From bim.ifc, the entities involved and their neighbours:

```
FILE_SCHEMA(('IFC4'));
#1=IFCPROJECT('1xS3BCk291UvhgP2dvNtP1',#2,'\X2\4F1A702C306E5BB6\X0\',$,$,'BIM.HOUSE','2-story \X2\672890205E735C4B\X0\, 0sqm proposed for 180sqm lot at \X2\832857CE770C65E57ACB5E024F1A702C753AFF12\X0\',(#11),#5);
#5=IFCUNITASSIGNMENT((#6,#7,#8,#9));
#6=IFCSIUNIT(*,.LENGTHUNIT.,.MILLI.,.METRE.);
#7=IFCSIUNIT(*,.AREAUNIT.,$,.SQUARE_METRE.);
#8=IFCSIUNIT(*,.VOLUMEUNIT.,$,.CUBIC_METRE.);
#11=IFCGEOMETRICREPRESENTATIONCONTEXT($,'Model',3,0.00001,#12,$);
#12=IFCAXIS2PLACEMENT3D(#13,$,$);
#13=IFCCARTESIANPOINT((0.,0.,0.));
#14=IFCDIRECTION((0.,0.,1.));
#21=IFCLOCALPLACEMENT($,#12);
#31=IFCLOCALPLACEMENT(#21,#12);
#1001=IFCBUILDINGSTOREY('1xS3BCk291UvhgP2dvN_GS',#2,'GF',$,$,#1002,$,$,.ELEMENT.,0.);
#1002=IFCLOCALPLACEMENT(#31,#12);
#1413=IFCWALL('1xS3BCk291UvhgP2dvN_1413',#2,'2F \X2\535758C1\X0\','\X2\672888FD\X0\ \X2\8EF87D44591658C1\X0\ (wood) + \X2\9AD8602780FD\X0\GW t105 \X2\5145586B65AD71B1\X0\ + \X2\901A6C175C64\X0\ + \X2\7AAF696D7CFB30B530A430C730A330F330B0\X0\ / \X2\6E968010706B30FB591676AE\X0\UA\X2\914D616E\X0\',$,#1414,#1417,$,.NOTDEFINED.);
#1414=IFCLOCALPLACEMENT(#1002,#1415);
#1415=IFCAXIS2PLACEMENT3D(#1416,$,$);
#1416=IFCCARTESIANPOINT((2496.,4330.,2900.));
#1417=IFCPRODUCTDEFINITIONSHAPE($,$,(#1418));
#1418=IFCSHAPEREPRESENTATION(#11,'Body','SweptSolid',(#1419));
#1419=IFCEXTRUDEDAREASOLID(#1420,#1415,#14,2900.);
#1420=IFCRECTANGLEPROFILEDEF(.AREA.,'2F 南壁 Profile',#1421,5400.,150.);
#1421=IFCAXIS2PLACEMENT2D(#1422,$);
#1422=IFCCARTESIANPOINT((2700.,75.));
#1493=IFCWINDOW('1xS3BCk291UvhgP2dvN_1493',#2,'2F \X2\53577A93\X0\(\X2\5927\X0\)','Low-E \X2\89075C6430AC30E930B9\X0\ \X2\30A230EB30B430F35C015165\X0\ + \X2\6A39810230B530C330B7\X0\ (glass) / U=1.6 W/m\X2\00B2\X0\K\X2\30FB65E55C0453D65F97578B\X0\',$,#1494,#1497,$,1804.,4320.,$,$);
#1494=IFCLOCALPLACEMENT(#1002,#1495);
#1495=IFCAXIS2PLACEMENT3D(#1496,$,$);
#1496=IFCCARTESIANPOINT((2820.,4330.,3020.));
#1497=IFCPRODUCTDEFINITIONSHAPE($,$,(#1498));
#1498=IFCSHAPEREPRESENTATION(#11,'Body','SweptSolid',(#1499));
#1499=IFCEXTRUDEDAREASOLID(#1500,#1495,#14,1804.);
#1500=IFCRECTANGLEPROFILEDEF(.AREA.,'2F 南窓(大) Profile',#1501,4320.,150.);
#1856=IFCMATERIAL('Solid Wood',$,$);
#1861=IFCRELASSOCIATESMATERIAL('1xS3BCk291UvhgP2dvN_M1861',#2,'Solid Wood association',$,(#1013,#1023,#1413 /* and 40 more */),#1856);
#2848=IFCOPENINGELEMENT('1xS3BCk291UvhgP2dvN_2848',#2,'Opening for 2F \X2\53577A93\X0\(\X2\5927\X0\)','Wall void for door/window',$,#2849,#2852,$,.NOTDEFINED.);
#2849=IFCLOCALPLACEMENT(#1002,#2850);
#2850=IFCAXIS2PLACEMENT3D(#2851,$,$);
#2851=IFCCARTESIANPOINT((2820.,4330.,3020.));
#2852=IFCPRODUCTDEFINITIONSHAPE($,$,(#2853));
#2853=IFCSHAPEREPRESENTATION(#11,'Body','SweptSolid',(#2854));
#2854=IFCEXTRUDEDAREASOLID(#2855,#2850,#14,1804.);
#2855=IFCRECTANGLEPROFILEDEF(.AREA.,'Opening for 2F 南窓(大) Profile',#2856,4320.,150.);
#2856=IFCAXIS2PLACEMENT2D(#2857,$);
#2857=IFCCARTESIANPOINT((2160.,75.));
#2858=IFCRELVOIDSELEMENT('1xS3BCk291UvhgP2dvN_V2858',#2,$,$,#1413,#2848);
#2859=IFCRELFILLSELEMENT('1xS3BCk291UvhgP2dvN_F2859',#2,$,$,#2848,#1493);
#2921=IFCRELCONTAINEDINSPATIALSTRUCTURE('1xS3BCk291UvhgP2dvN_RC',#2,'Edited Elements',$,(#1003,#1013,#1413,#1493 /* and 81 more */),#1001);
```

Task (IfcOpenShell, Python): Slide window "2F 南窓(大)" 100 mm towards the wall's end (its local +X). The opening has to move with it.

```python
import ifcopenshell
import ifcopenshell.api.geometry
import ifcopenshell.util.placement
import ifcopenshell.util.unit

model = ifcopenshell.open("bim.ifc")
unit_scale = ifcopenshell.util.unit.calculate_unit_scale(model)

window = model.by_id(1493)
opening = window.FillsVoids[0].RelatingOpeningElement
wall = opening.VoidsElements[0].RelatingBuildingElement

wall_matrix = ifcopenshell.util.placement.get_local_placement(wall.ObjectPlacement)
shift = wall_matrix[:3, 0] * 0.1 / unit_scale
before = ifcopenshell.util.placement.get_local_placement(window.ObjectPlacement)[:3, 3].copy()

# The window is not placed relative to its opening, so move both.
for product in (opening, window):
    matrix = ifcopenshell.util.placement.get_local_placement(product.ObjectPlacement)
    matrix[:3, 3] += shift
    ifcopenshell.api.geometry.edit_object_placement(model, product=product, matrix=matrix, is_si=False)

after = ifcopenshell.util.placement.get_local_placement(window.ObjectPlacement)[:3, 3]
print("window moved by", (after - before).round(3) + 0.0)

model.write("bim_rev.ifc")
```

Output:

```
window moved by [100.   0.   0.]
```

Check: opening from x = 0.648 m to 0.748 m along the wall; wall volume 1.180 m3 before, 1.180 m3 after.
